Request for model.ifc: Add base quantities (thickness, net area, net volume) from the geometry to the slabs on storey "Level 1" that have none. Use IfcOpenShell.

First a look at what the model holds.

```python
import ifcopenshell
import ifcopenshell.util.element
import ifcopenshell.util.unit

model = ifcopenshell.open("model.ifc")
print(model.schema)
for unit_type in ("LENGTHUNIT", "AREAUNIT", "VOLUMEUNIT"):
    print(unit_type, ifcopenshell.util.unit.calculate_unit_scale(model, unit_type))
storey = next(s for s in model.by_type("IfcBuildingStorey") if s.Name == "Level 1")
slabs = [e for e in ifcopenshell.util.element.get_decomposition(storey) if e.is_a("IfcSlab")]
for e in sorted(slabs, key=lambda e: e.id()):
    print(e.id(), e.is_a(), e.Name, list(ifcopenshell.util.element.get_psets(e, qtos_only=True)), sep=" | ")
```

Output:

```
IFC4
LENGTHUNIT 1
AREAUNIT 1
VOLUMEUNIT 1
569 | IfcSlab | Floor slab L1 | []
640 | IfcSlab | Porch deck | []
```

```python
import ifcopenshell
import ifcopenshell.api.pset
import ifcopenshell.geom
import ifcopenshell.util.element
import ifcopenshell.util.shape
import ifcopenshell.util.unit

model = ifcopenshell.open("model.ifc")
unit_scale = ifcopenshell.util.unit.calculate_unit_scale(model)
area_scale = ifcopenshell.util.unit.calculate_unit_scale(model, "AREAUNIT")
volume_scale = ifcopenshell.util.unit.calculate_unit_scale(model, "VOLUMEUNIT")
settings = ifcopenshell.geom.settings()

storey = next(s for s in model.by_type("IfcBuildingStorey") if s.Name == "Level 1")
slabs = [e for e in ifcopenshell.util.element.get_decomposition(storey) if e.is_a("IfcSlab")]

for e in sorted(slabs, key=lambda e: e.id()):
    if ifcopenshell.util.element.get_psets(e, qtos_only=True, should_inherit=False):
        continue
    # Geometry comes back in metres, in the element's own axes.
    shape = ifcopenshell.geom.create_shape(settings, e)
    values = {
        "Width": ifcopenshell.util.shape.get_z(shape.geometry) / unit_scale,
        "NetArea": ifcopenshell.util.shape.get_footprint_area(shape.geometry) / area_scale,
        "NetVolume": ifcopenshell.util.shape.get_volume(shape.geometry) / volume_scale,
    }
    qto = ifcopenshell.api.pset.add_qto(model, product=e, name="Qto_SlabBaseQuantities")
    ifcopenshell.api.pset.edit_qto(model, qto=qto, properties=values)
    print(e.id(), {k: round(v, 3) for k, v in values.items()})

model.write("model_v2.ifc")
```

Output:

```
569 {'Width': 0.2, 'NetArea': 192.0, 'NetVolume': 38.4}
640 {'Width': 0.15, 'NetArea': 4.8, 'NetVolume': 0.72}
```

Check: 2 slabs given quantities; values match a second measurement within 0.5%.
